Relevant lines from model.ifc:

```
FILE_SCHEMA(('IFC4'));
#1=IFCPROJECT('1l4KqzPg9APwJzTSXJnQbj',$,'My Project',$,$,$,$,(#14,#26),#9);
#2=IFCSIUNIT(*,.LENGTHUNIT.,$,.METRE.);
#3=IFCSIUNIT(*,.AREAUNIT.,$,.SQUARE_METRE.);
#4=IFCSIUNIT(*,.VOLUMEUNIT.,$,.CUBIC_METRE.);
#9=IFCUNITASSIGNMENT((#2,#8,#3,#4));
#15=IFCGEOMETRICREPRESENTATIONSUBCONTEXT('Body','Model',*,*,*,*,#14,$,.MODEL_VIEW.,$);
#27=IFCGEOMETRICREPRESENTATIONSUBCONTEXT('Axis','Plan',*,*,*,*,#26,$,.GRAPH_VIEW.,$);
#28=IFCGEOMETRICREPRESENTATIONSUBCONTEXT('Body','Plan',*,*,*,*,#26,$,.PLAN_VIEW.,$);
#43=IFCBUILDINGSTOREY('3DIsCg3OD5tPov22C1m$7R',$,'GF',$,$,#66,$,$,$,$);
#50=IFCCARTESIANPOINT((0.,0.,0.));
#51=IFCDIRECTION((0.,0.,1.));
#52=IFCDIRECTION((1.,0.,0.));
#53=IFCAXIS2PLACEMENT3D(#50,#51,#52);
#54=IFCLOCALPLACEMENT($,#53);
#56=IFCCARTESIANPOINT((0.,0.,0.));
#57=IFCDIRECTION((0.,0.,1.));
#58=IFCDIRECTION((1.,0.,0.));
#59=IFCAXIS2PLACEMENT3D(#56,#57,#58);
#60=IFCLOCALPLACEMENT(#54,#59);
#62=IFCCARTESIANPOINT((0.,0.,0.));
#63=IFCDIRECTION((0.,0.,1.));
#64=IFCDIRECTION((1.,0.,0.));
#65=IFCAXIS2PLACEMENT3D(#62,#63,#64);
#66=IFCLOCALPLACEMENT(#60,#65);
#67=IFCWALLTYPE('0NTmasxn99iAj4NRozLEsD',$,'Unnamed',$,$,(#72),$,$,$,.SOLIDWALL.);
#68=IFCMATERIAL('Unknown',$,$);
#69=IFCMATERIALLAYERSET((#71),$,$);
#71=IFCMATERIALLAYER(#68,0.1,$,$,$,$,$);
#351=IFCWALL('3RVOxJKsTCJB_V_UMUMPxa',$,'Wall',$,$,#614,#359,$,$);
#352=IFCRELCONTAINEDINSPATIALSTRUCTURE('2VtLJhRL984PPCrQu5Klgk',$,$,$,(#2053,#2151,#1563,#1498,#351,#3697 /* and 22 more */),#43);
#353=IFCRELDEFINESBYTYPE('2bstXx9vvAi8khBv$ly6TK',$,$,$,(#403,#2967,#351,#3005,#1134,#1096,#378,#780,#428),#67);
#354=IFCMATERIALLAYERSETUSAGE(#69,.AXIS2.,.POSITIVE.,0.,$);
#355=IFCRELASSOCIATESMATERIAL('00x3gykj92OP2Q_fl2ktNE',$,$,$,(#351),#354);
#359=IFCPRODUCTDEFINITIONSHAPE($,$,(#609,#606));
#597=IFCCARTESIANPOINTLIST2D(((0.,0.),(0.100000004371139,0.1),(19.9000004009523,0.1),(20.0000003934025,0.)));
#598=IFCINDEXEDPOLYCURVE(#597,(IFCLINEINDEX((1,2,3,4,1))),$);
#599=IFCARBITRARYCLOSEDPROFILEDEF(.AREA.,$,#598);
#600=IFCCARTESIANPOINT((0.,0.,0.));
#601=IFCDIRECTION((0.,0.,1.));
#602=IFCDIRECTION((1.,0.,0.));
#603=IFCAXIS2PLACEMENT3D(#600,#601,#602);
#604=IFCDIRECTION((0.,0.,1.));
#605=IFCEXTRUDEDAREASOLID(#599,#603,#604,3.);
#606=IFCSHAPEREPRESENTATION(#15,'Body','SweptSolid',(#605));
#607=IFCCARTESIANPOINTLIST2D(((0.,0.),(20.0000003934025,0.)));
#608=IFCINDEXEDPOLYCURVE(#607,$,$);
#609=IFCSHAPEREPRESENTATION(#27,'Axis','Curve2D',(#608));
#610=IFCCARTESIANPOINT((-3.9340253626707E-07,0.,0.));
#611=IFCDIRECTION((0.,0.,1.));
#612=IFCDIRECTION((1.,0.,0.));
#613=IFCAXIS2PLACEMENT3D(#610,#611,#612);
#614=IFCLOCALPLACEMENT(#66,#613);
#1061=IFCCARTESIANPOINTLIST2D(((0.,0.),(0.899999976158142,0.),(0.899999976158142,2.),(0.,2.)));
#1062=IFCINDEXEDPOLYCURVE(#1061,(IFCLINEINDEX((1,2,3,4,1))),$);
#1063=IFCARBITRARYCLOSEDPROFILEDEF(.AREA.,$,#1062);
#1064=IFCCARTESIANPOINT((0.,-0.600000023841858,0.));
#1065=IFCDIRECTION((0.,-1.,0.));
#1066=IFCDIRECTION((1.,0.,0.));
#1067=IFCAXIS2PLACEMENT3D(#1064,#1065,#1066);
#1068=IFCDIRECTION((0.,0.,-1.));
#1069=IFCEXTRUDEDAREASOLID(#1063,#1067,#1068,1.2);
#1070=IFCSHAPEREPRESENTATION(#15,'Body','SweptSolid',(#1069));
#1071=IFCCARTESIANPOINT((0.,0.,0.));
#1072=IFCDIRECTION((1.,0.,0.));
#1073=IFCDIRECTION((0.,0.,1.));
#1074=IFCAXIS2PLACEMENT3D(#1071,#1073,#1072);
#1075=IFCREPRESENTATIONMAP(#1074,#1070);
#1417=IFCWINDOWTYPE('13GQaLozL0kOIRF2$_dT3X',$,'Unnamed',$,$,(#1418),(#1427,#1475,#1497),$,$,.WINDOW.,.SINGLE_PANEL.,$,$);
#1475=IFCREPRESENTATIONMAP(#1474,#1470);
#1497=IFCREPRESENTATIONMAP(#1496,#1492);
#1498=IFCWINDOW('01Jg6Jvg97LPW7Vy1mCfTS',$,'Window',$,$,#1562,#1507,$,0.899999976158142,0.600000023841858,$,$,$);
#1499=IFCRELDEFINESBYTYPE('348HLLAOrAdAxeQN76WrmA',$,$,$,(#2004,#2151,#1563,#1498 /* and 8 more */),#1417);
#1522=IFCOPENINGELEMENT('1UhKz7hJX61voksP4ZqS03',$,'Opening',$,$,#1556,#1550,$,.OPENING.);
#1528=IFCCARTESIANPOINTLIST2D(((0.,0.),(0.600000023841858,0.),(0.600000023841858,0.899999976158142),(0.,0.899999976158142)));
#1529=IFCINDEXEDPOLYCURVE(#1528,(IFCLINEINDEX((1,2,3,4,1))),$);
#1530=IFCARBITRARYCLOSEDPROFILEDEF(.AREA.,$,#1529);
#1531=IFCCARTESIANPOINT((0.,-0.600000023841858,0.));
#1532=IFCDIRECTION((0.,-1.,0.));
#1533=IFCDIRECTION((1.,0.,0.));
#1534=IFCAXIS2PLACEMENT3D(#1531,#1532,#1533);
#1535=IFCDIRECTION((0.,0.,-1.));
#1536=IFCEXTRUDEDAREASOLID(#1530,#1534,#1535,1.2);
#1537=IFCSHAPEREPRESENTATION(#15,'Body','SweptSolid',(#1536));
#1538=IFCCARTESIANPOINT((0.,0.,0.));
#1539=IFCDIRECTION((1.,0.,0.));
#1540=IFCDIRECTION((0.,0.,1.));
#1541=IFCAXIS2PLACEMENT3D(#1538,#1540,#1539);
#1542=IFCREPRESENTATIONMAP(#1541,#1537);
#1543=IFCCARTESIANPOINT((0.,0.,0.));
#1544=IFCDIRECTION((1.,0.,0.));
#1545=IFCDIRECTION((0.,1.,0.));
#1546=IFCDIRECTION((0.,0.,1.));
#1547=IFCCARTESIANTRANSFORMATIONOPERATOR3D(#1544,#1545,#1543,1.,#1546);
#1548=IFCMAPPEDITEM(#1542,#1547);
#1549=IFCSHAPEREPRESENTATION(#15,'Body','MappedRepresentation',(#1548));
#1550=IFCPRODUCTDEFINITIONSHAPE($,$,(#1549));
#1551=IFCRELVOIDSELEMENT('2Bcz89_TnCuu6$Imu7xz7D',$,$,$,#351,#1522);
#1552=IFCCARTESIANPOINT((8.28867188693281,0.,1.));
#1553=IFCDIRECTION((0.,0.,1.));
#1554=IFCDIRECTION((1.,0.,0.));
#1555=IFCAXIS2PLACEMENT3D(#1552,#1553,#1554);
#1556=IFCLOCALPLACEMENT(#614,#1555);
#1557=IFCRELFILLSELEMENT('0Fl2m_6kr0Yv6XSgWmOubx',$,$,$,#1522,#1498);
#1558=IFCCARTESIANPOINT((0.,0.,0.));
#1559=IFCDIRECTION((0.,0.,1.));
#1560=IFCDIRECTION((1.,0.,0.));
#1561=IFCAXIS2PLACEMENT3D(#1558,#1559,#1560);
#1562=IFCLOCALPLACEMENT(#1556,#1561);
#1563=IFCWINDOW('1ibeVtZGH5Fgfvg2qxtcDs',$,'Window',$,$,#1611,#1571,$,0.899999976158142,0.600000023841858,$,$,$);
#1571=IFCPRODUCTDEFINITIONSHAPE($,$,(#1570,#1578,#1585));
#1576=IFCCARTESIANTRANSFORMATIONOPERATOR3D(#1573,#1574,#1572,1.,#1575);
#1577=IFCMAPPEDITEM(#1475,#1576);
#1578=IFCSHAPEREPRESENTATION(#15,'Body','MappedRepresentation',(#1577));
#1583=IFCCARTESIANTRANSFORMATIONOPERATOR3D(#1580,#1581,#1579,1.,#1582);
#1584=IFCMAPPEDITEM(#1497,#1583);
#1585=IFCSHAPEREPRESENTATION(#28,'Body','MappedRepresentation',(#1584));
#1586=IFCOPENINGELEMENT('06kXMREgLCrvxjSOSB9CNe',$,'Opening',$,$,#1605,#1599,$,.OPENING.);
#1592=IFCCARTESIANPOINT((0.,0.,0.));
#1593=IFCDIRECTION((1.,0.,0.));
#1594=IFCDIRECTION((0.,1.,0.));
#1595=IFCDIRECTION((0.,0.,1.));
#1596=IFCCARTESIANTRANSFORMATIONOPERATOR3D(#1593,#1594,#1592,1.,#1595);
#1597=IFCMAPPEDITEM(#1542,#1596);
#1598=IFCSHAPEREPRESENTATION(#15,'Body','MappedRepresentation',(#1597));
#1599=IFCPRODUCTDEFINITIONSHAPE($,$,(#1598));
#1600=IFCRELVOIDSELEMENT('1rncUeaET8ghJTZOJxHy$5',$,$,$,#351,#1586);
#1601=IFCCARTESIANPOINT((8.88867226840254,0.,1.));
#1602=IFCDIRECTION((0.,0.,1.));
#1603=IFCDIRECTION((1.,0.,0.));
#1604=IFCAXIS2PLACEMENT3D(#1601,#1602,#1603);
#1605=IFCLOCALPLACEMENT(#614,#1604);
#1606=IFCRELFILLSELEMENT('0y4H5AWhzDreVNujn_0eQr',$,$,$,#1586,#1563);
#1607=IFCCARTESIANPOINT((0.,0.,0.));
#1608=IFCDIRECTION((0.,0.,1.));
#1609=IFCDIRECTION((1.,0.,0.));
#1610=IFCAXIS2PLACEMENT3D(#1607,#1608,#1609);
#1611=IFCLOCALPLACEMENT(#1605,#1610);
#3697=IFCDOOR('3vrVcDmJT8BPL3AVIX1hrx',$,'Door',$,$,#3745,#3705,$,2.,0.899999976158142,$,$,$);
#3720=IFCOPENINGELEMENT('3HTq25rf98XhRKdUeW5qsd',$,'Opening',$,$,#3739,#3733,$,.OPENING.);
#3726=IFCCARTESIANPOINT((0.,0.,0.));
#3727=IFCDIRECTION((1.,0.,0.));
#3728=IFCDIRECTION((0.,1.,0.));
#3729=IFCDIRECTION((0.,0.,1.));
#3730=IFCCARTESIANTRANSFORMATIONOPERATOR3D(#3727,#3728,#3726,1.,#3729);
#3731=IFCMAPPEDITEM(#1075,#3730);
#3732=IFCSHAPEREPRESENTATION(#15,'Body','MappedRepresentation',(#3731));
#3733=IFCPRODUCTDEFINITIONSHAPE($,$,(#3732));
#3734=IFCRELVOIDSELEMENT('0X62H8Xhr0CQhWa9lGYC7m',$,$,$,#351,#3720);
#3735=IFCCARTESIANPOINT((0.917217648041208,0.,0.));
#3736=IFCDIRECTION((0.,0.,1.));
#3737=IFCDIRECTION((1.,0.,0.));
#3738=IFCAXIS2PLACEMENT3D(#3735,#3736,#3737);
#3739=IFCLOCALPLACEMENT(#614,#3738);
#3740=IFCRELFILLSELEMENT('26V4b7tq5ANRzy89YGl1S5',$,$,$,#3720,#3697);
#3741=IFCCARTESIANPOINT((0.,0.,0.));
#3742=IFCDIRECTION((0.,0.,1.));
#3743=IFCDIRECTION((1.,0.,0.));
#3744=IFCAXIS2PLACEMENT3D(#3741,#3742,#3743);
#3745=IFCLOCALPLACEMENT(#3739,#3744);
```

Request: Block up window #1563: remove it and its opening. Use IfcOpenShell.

```python
import ifcopenshell
import ifcopenshell.api.feature
import ifcopenshell.api.root
import ifcopenshell.geom
import ifcopenshell.util.shape

model = ifcopenshell.open("model.ifc")
settings = ifcopenshell.geom.settings()


def volume(element):
    """Net volume in cubic metres, openings subtracted."""
    shape = ifcopenshell.geom.create_shape(settings, element)
    return ifcopenshell.util.shape.get_volume(shape.geometry)


window = model.by_guid("1ibeVtZGH5Fgfvg2qxtcDs")
opening = window.FillsVoids[0].RelatingOpeningElement
wall = opening.VoidsElements[0].RelatingBuildingElement
before = volume(wall)

ifcopenshell.api.root.remove_product(model, product=window)
ifcopenshell.api.feature.remove_feature(model, feature=opening)

after = volume(wall)

print(f"wall volume {before:.3f} -> {after:.3f} m3")

model.write("model_updated.ifc")
```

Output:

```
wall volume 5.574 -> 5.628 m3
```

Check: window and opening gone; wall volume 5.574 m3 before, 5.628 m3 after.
